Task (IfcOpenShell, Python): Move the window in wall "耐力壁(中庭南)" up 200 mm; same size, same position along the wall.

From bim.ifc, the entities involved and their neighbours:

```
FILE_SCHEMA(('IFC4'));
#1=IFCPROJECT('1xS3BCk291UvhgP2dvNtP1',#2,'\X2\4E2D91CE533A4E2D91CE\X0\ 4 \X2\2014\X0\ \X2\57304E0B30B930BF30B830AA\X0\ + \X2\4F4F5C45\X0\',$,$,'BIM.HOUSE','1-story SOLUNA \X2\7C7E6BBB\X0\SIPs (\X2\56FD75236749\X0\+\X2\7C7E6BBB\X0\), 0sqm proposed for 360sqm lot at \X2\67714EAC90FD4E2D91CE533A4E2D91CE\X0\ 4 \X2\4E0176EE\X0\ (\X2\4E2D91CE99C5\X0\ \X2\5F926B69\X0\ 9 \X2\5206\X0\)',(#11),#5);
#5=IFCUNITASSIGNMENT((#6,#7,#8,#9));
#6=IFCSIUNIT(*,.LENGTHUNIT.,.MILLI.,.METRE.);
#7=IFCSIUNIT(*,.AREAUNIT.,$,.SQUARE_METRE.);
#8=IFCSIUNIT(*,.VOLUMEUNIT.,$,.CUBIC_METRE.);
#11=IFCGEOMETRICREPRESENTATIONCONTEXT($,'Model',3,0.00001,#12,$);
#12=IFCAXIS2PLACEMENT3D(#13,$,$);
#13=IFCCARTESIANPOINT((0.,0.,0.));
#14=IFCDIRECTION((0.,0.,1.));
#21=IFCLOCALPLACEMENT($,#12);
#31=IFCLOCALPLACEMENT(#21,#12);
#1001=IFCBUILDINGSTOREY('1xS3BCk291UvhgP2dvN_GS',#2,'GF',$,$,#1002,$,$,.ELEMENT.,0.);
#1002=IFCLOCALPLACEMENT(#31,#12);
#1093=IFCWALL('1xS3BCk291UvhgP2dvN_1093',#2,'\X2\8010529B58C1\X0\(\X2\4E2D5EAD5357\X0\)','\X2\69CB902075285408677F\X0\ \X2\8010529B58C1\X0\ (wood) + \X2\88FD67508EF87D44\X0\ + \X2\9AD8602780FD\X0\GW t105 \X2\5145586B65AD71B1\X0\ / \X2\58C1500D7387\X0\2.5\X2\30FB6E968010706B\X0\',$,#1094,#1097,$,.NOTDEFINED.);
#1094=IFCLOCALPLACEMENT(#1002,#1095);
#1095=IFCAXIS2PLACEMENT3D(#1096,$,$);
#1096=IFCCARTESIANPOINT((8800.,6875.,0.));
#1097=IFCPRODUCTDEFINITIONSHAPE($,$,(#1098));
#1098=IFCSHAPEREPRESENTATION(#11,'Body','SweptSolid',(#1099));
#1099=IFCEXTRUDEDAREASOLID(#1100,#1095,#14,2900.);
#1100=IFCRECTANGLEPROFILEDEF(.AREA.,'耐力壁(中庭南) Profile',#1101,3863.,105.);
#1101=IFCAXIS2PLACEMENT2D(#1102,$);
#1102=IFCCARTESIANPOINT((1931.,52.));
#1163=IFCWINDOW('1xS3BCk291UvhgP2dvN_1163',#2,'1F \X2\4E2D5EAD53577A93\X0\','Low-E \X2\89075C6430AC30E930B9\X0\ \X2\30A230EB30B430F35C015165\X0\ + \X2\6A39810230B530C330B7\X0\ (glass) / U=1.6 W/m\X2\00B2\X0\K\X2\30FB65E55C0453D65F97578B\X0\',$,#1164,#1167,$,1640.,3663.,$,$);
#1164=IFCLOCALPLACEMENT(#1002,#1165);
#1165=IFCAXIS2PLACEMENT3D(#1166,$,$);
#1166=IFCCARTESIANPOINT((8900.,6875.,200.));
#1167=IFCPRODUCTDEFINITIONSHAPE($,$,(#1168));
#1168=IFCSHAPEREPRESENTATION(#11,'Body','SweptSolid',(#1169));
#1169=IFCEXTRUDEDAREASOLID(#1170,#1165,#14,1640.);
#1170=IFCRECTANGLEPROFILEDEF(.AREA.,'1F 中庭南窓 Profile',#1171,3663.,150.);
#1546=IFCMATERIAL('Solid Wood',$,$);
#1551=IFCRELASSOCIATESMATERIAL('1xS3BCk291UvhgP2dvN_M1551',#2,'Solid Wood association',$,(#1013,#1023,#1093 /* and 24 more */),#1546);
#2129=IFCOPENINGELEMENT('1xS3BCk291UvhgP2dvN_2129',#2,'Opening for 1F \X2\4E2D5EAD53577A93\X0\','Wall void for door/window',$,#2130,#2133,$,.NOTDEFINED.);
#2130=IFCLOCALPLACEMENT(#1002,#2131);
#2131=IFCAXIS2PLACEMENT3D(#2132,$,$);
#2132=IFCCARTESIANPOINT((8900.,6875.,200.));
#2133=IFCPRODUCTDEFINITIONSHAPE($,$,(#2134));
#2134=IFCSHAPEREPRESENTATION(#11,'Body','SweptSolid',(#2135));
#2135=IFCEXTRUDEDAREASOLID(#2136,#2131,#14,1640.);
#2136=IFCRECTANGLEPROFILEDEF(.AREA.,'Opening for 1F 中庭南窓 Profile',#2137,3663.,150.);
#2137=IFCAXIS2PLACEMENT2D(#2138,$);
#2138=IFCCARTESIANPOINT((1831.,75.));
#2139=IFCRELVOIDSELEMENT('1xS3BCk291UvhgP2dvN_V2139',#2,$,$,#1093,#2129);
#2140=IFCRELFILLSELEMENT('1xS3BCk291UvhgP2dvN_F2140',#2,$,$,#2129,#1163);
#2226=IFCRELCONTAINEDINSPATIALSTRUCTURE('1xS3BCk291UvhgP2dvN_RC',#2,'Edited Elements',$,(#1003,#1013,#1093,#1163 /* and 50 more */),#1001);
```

```python
import numpy as np
import ifcopenshell
import ifcopenshell.api.geometry
import ifcopenshell.util.placement
import ifcopenshell.util.unit

model = ifcopenshell.open("bim.ifc")
unit_scale = ifcopenshell.util.unit.calculate_unit_scale(model)

window = model.by_id(1163)
opening = window.FillsVoids[0].RelatingOpeningElement
dz = 0.2 / unit_scale

shift = np.array([0.0, 0.0, dz])
# The window is not placed relative to its opening, so move both.
for product in (opening, window):
    matrix = ifcopenshell.util.placement.get_local_placement(product.ObjectPlacement)
    matrix[:3, 3] += shift
    ifcopenshell.api.geometry.edit_object_placement(model, product=product, matrix=matrix, is_si=False)

print(f"moved by {dz * unit_scale:+.3f} m")

model.write("bim-out.ifc")
```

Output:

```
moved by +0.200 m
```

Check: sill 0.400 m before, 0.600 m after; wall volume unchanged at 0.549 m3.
